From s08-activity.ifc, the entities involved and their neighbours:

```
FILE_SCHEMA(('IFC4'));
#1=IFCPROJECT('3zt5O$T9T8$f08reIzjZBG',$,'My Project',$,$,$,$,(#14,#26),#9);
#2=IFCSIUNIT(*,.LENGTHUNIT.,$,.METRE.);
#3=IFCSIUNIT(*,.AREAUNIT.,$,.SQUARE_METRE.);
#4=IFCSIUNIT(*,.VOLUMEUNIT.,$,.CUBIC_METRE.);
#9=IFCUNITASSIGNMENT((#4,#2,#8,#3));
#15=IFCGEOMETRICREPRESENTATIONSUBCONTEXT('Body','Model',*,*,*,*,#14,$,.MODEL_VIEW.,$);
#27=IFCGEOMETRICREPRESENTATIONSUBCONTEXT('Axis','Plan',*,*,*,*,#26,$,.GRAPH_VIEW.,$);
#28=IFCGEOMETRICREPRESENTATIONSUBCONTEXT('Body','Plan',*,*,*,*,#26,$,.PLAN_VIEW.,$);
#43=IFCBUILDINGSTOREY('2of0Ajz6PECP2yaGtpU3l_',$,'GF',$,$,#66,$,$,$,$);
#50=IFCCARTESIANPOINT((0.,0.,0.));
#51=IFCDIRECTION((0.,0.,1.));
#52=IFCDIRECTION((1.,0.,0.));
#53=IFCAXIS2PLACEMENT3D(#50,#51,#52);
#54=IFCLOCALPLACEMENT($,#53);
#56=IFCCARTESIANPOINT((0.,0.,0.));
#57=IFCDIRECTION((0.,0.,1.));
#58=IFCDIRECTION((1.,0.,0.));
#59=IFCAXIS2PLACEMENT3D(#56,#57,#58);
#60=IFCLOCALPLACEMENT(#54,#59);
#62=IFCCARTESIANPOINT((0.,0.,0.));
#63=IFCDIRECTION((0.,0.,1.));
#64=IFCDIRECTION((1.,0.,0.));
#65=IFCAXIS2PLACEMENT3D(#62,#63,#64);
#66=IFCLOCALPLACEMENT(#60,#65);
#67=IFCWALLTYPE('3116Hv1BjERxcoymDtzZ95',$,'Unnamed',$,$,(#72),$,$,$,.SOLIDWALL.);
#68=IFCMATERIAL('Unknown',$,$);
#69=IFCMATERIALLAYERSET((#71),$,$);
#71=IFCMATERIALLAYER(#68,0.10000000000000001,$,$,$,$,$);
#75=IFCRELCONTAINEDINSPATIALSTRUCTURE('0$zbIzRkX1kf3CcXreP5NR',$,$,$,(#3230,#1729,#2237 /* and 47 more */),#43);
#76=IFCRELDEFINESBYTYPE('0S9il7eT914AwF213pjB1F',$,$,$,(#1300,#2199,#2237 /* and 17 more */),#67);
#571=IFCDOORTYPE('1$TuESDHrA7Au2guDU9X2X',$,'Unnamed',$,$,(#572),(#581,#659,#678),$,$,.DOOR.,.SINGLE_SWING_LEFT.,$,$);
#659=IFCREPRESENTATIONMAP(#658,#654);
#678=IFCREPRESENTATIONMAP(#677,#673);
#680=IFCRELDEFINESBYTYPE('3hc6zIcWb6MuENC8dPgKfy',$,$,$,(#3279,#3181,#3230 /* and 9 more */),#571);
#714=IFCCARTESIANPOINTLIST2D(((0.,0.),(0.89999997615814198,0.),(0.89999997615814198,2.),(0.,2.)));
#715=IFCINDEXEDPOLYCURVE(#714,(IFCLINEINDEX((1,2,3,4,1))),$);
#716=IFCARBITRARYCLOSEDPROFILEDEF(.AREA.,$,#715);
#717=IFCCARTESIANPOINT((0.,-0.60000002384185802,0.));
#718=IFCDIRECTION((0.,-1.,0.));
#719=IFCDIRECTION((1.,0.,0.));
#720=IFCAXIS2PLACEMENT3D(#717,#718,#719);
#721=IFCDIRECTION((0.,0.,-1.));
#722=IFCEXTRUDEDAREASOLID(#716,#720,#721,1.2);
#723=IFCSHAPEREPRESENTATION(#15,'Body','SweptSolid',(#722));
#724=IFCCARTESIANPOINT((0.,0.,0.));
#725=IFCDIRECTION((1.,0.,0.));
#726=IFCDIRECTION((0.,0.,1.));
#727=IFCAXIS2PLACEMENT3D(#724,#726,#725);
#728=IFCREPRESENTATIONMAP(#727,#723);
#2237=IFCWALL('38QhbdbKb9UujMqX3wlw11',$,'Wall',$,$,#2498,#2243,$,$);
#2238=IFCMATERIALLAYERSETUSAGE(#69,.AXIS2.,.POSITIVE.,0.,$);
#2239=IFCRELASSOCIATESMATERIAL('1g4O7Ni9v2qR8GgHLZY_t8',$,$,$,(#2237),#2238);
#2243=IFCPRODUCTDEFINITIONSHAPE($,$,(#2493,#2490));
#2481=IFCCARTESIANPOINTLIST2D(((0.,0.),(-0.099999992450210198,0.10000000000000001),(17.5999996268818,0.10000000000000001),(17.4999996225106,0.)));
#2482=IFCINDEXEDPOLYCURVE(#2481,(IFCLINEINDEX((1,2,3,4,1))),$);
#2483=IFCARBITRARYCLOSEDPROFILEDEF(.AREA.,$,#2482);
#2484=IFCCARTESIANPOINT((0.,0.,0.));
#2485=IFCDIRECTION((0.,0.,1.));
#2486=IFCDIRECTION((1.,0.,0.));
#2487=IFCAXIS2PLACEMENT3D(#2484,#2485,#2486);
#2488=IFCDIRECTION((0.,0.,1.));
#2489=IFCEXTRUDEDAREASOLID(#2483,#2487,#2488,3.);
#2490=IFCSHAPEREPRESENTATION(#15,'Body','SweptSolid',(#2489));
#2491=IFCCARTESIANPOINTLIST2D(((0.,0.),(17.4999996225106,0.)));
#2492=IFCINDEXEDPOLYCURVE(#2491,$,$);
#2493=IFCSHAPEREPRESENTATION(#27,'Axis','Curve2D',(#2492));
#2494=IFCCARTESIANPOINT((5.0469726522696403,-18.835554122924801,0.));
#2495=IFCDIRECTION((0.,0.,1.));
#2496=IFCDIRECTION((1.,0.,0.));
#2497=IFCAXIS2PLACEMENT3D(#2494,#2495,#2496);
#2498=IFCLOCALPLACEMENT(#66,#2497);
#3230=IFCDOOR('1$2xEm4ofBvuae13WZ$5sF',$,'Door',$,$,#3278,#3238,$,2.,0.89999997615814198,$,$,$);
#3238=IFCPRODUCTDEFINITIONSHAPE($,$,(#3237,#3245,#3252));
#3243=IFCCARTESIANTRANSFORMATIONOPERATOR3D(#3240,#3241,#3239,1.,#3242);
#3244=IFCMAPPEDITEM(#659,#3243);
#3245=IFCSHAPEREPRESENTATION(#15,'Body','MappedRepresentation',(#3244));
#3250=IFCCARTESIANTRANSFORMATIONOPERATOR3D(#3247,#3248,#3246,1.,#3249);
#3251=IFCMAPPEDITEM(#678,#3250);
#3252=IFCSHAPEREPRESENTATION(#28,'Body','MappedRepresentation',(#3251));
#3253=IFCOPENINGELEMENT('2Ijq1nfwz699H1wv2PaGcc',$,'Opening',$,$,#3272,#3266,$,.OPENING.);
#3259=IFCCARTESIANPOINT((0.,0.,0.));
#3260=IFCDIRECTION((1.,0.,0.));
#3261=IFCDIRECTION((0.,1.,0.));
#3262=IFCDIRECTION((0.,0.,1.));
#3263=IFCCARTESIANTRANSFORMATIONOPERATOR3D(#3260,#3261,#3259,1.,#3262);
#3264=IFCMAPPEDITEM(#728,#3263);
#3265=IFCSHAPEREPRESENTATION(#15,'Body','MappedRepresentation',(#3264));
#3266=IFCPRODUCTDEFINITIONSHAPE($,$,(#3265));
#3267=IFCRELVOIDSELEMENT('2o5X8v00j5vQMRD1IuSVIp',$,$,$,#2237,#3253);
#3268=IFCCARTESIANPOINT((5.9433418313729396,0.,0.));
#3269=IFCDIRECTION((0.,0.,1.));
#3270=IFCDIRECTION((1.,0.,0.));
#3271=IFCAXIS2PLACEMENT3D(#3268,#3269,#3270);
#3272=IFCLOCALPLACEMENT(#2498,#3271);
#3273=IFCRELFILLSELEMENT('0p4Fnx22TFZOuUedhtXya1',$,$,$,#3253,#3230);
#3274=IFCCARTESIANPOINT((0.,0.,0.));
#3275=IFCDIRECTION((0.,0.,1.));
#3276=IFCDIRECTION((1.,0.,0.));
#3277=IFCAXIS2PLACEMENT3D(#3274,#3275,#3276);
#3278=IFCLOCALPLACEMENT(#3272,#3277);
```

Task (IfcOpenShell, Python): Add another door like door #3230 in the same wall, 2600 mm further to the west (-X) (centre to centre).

```python
import ifcopenshell
import ifcopenshell.api.feature
import ifcopenshell.api.geometry
import ifcopenshell.api.root
import ifcopenshell.geom
import ifcopenshell.util.element
import ifcopenshell.util.placement
import ifcopenshell.util.shape

model = ifcopenshell.open("s08-activity.ifc")
settings = ifcopenshell.geom.settings()


def volume(element):
    """Net volume in cubic metres, openings subtracted."""
    shape = ifcopenshell.geom.create_shape(settings, element)
    return ifcopenshell.util.shape.get_volume(shape.geometry)


door = model.by_id(3230)
opening = door.FillsVoids[0].RelatingOpeningElement
wall = opening.VoidsElements[0].RelatingBuildingElement
before = volume(wall)
shift = ifcopenshell.util.placement.get_local_placement(wall.ObjectPlacement)[:3, 0] * -2.6

# copy_class copies the void relationship, type, container and properties, but no geometry.
new_opening = ifcopenshell.api.root.copy_class(model, product=opening)
new_opening.Representation = ifcopenshell.util.element.copy_deep(
    model, opening.Representation, exclude=["IfcGeometricRepresentationContext", "IfcRepresentationMap"]
)
new_door = ifcopenshell.api.root.copy_class(model, product=door)
new_door.Representation = ifcopenshell.util.element.copy_deep(
    model, door.Representation, exclude=["IfcGeometricRepresentationContext", "IfcRepresentationMap"]
)
ifcopenshell.api.feature.add_filling(model, opening=new_opening, element=new_door)

for old, new in ((opening, new_opening), (door, new_door)):
    matrix = ifcopenshell.util.placement.get_local_placement(old.ObjectPlacement)
    matrix[:3, 3] += shift
    ifcopenshell.api.geometry.edit_object_placement(model, product=new, matrix=matrix, is_si=False)

after = volume(wall)

print(f"wall volume {before:.3f} -> {after:.3f} m3")

model.write("s08-activity_updated.ifc")
```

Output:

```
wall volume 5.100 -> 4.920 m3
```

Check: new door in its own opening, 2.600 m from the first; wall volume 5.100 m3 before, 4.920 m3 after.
